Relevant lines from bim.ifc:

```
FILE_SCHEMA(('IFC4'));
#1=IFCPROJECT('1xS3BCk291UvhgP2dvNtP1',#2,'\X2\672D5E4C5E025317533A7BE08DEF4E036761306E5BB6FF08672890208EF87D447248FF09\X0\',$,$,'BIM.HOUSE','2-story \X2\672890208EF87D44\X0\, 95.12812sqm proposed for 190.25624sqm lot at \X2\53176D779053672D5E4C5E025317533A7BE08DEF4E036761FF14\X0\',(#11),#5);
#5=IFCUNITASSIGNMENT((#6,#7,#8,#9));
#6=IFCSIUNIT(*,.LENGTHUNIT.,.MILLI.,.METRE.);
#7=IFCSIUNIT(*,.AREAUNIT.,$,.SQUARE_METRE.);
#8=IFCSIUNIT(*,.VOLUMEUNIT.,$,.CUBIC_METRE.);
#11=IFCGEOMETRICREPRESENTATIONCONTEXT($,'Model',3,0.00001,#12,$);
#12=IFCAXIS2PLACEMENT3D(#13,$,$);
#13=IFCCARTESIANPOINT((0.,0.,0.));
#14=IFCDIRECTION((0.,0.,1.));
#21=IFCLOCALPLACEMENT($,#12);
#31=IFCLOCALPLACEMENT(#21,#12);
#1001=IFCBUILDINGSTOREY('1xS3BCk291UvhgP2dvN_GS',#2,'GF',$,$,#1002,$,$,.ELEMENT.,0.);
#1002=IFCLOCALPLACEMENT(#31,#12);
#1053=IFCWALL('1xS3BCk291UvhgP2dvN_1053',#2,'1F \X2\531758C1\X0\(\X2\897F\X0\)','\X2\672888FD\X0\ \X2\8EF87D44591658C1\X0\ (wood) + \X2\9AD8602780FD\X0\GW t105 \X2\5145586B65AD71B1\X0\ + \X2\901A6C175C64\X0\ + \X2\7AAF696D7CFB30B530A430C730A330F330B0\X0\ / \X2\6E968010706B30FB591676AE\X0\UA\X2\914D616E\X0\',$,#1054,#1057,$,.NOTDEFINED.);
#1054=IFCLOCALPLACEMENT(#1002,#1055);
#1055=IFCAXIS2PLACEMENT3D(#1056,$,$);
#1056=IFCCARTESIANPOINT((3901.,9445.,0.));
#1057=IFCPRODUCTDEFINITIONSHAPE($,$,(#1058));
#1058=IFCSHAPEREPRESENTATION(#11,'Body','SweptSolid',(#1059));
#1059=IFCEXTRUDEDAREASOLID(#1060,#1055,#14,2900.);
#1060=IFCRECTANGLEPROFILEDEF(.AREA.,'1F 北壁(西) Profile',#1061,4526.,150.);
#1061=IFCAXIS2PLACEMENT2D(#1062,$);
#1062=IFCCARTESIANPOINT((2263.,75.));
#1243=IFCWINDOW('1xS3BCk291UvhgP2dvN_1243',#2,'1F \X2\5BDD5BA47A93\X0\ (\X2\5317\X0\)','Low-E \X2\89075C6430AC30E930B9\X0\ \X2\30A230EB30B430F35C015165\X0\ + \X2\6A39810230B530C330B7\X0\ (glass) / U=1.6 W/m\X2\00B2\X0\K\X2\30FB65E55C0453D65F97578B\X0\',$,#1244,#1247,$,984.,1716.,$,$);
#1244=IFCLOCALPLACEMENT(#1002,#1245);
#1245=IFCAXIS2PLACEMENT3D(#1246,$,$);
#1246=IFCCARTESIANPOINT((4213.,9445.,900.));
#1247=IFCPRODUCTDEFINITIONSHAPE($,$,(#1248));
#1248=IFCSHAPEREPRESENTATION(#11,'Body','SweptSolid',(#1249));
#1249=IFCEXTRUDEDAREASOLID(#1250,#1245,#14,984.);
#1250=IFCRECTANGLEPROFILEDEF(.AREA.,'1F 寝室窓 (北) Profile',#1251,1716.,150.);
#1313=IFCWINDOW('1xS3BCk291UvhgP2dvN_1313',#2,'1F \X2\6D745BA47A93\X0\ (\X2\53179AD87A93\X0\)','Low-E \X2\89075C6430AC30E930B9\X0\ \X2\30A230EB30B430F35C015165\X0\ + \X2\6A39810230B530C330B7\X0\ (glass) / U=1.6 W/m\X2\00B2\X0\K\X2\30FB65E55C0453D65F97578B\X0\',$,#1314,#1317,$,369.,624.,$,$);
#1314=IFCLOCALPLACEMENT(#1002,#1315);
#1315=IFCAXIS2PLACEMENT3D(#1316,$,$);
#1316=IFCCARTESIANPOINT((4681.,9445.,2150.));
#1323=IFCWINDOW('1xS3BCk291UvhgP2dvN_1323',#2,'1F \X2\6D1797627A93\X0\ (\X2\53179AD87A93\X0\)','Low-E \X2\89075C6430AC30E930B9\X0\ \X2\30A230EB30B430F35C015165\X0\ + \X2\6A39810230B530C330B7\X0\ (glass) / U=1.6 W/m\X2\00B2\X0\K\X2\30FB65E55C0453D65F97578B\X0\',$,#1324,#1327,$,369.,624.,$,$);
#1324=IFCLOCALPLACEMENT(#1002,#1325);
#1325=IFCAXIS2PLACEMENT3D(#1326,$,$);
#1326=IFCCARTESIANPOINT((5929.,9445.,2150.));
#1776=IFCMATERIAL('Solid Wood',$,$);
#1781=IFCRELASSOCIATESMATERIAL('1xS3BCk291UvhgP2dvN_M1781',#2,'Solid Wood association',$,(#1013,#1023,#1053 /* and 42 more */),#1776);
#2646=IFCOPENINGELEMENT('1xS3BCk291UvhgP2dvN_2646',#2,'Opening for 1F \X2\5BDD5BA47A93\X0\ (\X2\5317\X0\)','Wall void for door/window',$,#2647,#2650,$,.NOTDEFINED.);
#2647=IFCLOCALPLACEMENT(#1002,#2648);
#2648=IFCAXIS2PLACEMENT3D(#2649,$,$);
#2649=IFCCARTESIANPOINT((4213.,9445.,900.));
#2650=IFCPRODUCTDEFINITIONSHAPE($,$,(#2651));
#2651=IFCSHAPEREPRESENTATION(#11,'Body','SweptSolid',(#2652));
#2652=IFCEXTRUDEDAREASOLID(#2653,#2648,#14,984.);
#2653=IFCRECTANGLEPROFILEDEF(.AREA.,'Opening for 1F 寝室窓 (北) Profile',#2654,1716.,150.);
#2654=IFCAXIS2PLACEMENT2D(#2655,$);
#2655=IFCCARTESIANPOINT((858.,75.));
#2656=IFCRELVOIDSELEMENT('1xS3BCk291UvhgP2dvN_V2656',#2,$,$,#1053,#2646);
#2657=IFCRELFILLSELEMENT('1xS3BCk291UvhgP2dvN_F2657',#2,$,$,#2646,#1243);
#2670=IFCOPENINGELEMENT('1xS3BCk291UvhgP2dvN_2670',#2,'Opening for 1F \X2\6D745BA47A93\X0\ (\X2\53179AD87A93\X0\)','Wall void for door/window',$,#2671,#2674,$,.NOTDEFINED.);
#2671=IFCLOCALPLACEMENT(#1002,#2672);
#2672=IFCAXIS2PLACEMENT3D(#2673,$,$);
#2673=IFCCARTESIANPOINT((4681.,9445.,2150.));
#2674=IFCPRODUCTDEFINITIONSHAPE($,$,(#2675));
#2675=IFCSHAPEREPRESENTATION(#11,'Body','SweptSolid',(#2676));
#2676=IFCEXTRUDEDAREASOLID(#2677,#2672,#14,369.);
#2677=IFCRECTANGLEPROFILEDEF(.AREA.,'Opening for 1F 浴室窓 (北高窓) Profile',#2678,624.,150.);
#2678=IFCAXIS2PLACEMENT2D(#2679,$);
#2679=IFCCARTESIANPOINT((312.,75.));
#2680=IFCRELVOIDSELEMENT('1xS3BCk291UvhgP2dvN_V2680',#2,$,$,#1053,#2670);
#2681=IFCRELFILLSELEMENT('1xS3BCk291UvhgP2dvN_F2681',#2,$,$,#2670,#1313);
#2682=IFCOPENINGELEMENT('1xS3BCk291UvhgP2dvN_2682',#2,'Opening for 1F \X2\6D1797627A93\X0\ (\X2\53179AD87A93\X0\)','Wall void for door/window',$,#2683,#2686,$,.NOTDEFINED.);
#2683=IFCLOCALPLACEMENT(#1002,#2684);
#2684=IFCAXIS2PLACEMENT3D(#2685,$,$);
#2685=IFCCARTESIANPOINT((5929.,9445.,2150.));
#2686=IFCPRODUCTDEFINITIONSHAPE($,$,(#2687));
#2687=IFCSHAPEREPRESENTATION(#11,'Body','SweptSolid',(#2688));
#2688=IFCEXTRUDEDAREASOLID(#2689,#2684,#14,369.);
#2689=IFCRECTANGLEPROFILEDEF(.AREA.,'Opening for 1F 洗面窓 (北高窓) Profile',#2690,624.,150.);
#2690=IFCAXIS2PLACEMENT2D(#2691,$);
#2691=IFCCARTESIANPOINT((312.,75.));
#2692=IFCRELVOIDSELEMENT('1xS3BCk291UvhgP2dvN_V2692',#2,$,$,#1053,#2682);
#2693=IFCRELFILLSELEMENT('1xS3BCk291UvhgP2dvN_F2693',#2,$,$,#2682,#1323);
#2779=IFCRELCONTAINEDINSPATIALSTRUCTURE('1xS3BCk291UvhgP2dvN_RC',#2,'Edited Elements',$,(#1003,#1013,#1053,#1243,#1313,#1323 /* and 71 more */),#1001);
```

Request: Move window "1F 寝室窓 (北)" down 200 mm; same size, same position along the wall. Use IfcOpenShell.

```python
import numpy as np
import ifcopenshell
import ifcopenshell.api.geometry
import ifcopenshell.util.placement
import ifcopenshell.util.unit

model = ifcopenshell.open("bim.ifc")
unit_scale = ifcopenshell.util.unit.calculate_unit_scale(model)

window = model.by_guid("1xS3BCk291UvhgP2dvN_1243")
opening = window.FillsVoids[0].RelatingOpeningElement
dz = -0.2 / unit_scale

shift = np.array([0.0, 0.0, dz])
# The window is not placed relative to its opening, so move both.
for product in (opening, window):
    matrix = ifcopenshell.util.placement.get_local_placement(product.ObjectPlacement)
    matrix[:3, 3] += shift
    ifcopenshell.api.geometry.edit_object_placement(model, product=product, matrix=matrix, is_si=False)

print(f"moved by {dz * unit_scale:+.3f} m")

model.write("bim_v2.ifc")
```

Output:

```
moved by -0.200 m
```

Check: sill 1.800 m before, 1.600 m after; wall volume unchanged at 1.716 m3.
